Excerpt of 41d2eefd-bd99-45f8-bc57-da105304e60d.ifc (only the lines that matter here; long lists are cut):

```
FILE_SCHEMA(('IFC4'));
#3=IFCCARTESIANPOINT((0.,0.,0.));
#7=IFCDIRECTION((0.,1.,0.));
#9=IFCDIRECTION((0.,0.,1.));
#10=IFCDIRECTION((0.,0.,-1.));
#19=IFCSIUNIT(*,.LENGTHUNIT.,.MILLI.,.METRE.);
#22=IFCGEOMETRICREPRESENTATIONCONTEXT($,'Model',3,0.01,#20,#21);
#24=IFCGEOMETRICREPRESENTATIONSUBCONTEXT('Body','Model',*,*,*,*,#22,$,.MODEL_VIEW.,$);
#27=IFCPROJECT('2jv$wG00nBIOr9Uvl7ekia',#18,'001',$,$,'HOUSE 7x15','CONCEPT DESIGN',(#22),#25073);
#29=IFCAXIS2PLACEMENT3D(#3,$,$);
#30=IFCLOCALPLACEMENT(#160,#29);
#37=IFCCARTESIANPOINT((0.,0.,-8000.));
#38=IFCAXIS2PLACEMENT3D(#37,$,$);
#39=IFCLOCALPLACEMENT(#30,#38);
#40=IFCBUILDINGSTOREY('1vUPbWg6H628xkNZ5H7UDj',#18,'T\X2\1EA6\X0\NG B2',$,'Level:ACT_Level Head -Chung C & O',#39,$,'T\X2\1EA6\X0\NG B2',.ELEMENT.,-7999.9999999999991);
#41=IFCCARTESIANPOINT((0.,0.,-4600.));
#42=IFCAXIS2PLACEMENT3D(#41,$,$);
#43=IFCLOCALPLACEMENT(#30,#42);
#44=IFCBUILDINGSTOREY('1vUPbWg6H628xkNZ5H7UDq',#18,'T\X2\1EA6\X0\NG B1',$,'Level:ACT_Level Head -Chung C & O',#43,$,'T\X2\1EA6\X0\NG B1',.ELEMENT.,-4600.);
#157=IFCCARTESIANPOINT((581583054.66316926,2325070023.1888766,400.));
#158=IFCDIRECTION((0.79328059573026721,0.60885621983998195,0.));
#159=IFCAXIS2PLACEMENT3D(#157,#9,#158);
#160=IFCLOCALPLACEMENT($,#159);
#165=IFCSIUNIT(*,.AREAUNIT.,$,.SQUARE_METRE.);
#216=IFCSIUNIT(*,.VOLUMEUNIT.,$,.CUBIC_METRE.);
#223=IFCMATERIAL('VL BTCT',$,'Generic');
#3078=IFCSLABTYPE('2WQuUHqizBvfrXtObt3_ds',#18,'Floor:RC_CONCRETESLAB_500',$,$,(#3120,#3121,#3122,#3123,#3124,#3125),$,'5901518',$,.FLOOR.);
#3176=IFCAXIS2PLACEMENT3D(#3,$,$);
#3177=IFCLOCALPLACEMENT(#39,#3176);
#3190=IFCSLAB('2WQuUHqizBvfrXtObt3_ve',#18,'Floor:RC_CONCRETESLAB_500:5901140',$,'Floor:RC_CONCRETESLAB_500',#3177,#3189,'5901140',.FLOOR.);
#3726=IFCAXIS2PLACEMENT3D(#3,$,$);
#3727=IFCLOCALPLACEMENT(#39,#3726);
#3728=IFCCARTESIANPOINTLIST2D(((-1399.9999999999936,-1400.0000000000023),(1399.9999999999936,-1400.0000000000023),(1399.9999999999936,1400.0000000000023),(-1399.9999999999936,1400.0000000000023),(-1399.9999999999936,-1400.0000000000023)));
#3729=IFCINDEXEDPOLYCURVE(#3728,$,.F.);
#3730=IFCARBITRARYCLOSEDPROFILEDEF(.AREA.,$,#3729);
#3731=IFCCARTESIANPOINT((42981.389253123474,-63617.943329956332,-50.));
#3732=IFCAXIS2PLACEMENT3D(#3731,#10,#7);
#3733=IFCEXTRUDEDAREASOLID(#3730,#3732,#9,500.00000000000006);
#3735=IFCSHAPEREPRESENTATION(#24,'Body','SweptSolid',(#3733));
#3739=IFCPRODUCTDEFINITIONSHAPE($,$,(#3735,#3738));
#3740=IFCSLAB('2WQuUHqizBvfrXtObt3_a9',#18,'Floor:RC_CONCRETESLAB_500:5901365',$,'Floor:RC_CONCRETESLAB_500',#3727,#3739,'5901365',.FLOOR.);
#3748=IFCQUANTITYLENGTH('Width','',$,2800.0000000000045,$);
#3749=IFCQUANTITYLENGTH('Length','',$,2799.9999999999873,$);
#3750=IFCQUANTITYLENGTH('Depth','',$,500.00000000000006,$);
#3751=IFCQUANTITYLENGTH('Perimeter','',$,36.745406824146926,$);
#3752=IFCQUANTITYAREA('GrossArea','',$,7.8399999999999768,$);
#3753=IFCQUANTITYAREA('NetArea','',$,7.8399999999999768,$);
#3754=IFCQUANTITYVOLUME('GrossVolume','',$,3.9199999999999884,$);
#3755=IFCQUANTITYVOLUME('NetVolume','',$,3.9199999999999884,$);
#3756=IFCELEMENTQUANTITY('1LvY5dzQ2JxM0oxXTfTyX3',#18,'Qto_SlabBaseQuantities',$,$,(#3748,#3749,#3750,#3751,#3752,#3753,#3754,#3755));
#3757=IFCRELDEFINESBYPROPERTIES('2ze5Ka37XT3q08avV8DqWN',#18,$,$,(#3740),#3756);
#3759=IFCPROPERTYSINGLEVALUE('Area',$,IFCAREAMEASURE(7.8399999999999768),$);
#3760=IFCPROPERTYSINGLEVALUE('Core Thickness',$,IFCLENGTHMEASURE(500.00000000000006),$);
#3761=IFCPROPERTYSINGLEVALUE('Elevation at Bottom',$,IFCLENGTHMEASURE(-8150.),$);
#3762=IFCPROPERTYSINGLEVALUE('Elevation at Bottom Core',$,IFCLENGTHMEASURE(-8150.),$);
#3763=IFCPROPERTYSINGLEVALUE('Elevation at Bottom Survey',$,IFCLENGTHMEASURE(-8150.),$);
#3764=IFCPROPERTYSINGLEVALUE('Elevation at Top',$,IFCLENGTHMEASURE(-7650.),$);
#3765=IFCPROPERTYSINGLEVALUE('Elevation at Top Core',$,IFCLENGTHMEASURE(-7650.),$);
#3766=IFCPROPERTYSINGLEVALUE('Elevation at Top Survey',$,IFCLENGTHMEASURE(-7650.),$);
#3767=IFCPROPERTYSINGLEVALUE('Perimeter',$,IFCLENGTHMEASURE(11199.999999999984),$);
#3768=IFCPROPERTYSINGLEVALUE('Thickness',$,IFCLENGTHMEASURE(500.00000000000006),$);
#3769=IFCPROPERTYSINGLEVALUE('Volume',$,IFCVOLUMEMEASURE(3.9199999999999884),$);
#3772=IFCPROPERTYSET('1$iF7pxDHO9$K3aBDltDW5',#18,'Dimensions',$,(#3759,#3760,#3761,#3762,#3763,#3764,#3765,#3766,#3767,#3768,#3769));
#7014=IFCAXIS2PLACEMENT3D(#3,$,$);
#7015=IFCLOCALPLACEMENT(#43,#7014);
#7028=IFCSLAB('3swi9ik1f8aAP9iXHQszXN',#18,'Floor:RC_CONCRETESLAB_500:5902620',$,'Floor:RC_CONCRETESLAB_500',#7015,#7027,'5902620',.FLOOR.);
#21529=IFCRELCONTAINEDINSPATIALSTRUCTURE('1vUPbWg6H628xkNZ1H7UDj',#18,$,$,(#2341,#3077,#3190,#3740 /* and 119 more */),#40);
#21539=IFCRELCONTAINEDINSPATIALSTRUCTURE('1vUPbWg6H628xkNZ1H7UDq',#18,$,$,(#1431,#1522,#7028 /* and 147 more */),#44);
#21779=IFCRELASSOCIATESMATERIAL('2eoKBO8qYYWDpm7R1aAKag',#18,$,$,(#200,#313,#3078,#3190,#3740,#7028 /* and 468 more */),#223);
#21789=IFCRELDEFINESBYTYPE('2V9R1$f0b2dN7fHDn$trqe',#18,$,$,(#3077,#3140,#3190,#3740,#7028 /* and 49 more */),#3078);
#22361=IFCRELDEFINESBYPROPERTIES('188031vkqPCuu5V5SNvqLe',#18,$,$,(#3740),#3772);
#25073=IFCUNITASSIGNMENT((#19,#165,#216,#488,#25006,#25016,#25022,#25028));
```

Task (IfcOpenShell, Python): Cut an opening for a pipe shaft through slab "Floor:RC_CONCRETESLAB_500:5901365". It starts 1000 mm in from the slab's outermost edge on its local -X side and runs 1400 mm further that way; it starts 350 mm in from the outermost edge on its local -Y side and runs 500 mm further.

```python
import numpy as np
import ifcopenshell
import ifcopenshell.api.feature
import ifcopenshell.api.geometry
import ifcopenshell.api.pset
import ifcopenshell.api.root
import ifcopenshell.geom
import ifcopenshell.util.element
import ifcopenshell.util.placement
import ifcopenshell.util.representation
import ifcopenshell.util.shape
import ifcopenshell.util.unit

model = ifcopenshell.open("41d2eefd-bd99-45f8-bc57-da105304e60d.ifc")
unit_scale = ifcopenshell.util.unit.calculate_unit_scale(model)
area_scale = ifcopenshell.util.unit.calculate_unit_scale(model, "AREAUNIT")
volume_scale = ifcopenshell.util.unit.calculate_unit_scale(model, "VOLUMEUNIT")
settings = ifcopenshell.geom.settings()


def volume(element):
    """Net volume in cubic metres, openings subtracted."""
    shape = ifcopenshell.geom.create_shape(settings, element)
    return ifcopenshell.util.shape.get_volume(shape.geometry)


slab = model.by_guid("2WQuUHqizBvfrXtObt3_a9")
before = volume(slab)

# Extent in the slab's own axes, in metres. The edges named are its -X and -Y sides.
slab_shape = ifcopenshell.geom.create_shape(settings, slab)
vertices = ifcopenshell.util.shape.get_vertices(slab_shape.geometry)
x_min, y_min, bottom = vertices.min(axis=0)
top = vertices[:, 2].max()

opening = ifcopenshell.api.root.create_entity(model, ifc_class="IfcOpeningElement", name="Pipe shaft opening", predefined_type="OPENING")
context = ifcopenshell.util.representation.get_context(model, "Model", "Body", "MODEL_VIEW")
width, depth = 1.4, 0.5
outline = [(0.0, 0.0), (width, 0.0), (width, depth), (0.0, depth), (0.0, 0.0)]
# Overshoot both faces by 50 mm so the cut is clean.
shape = ifcopenshell.api.geometry.add_slab_representation(
    model, context=context, depth=top - bottom + 0.1, polyline=outline
)
ifcopenshell.api.geometry.assign_representation(model, product=opening, representation=shape)

matrix = ifcopenshell.util.placement.get_local_placement(slab.ObjectPlacement)
matrix[:, 3] = matrix @ np.append(np.array([x_min + 1, y_min + 0.35, bottom - 0.05]) / unit_scale, 1.0)
ifcopenshell.api.geometry.edit_object_placement(model, product=opening, matrix=matrix, is_si=False)
ifcopenshell.api.feature.add_feature(model, feature=opening, element=slab)

after = volume(slab)

# Update the slab's stored quantities.
qto = model.by_id(ifcopenshell.util.element.get_pset(slab, "Qto_SlabBaseQuantities", should_inherit=False)["id"])
ifcopenshell.api.pset.edit_qto(model, qto=qto, properties={
    "NetArea": after / (top - bottom) / area_scale,
    "NetVolume": after / volume_scale,
})
pset = model.by_id(ifcopenshell.util.element.get_pset(slab, "Dimensions", should_inherit=False)["id"])
ifcopenshell.api.pset.edit_pset(model, pset=pset, properties={
    "Area": model.create_entity("IfcAreaMeasure", after / (top - bottom) / area_scale),
    "Volume": model.create_entity("IfcVolumeMeasure", after / volume_scale),
})

print(f"slab volume {before:.3f} -> {after:.3f} m3")

model.write("41d2eefd-bd99-45f8-bc57-da105304e60d_rev.ifc")
```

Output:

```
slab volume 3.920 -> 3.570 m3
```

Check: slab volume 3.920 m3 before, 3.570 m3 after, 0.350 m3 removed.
